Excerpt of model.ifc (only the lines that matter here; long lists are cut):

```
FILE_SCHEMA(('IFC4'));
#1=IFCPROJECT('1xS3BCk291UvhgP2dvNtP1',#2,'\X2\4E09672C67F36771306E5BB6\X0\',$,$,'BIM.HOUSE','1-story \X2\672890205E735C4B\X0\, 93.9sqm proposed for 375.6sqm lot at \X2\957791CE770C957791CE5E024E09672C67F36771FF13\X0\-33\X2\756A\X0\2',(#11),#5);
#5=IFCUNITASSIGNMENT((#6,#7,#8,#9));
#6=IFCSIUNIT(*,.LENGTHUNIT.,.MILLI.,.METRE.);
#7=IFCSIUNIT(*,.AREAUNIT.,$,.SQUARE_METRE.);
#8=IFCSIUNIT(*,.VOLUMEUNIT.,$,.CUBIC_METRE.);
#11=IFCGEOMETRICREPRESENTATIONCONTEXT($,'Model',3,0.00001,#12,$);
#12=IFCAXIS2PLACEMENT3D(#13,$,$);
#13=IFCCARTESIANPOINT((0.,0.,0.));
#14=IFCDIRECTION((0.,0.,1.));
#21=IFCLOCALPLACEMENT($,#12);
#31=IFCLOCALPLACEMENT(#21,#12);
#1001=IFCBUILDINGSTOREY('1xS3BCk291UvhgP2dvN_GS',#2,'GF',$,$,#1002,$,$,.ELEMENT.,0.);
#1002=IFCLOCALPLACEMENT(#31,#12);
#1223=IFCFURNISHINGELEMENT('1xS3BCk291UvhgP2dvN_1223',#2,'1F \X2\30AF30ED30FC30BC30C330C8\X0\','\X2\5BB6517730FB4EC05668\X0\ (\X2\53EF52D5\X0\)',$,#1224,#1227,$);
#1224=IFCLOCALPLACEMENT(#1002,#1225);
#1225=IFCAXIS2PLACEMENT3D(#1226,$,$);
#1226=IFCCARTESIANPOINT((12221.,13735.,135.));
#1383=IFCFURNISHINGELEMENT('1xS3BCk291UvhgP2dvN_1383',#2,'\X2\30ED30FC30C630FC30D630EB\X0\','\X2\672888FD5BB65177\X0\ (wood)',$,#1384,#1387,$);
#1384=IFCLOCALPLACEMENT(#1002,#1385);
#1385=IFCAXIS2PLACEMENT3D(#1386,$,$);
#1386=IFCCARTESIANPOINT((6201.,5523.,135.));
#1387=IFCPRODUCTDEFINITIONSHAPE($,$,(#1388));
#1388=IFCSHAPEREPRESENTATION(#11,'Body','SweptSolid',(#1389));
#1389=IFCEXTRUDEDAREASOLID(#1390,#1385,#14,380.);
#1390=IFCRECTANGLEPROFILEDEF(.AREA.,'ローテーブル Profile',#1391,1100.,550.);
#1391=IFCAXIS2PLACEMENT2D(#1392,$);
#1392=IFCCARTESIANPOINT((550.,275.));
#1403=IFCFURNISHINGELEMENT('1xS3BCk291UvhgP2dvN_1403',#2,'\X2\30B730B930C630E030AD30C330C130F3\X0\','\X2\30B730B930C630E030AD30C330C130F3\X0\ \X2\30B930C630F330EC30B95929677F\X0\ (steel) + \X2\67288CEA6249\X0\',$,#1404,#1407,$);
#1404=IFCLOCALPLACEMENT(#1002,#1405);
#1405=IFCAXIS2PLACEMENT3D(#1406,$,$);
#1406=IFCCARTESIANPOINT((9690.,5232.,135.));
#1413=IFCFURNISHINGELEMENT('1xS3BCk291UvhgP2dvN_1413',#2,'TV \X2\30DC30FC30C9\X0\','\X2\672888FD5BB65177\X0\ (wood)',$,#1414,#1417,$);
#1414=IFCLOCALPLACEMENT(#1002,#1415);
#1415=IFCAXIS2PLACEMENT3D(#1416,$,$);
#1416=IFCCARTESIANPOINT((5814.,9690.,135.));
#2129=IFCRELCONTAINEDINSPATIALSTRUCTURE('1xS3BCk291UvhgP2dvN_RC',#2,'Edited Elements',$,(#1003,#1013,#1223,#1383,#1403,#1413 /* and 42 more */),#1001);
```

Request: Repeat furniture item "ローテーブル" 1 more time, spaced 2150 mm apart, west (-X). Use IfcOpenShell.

```python
import numpy as np
import ifcopenshell
import ifcopenshell.api.geometry
import ifcopenshell.api.root
import ifcopenshell.util.element
import ifcopenshell.util.placement
import ifcopenshell.util.unit

model = ifcopenshell.open("model.ifc")
unit_scale = ifcopenshell.util.unit.calculate_unit_scale(model)


def reuse_history(source, copy):
    """copy_class also copies each property set's owner history, people and application; keep the originals."""
    for rel in copy.IsDefinedBy:
        if rel.is_a("IfcRelDefinesByProperties") and (history := rel.RelatingPropertyDefinition.OwnerHistory):
            rel.RelatingPropertyDefinition.OwnerHistory = source.OwnerHistory
            ifcopenshell.util.element.remove_deep2(model, history)


source = model.by_guid("1xS3BCk291UvhgP2dvN_1383")
base = ifcopenshell.util.placement.get_local_placement(source.ObjectPlacement)
step = np.array([-1.0, 0.0, 0.0]) * 2.15 / unit_scale

for i in range(1, 2):
    copy = ifcopenshell.api.root.copy_class(model, product=source)
    copy.Representation = ifcopenshell.util.element.copy_deep(
        model, source.Representation, exclude=["IfcGeometricRepresentationContext", "IfcRepresentationMap"]
    )
    reuse_history(source, copy)
    matrix = base.copy()
    matrix[:3, 3] += i * step
    print("added at", matrix[:3, 3].round(3) + 0.0)
    ifcopenshell.api.geometry.edit_object_placement(model, product=copy, matrix=matrix, is_si=False)

model.write("model_edited.ifc")
```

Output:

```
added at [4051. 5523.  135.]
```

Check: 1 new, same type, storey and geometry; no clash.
